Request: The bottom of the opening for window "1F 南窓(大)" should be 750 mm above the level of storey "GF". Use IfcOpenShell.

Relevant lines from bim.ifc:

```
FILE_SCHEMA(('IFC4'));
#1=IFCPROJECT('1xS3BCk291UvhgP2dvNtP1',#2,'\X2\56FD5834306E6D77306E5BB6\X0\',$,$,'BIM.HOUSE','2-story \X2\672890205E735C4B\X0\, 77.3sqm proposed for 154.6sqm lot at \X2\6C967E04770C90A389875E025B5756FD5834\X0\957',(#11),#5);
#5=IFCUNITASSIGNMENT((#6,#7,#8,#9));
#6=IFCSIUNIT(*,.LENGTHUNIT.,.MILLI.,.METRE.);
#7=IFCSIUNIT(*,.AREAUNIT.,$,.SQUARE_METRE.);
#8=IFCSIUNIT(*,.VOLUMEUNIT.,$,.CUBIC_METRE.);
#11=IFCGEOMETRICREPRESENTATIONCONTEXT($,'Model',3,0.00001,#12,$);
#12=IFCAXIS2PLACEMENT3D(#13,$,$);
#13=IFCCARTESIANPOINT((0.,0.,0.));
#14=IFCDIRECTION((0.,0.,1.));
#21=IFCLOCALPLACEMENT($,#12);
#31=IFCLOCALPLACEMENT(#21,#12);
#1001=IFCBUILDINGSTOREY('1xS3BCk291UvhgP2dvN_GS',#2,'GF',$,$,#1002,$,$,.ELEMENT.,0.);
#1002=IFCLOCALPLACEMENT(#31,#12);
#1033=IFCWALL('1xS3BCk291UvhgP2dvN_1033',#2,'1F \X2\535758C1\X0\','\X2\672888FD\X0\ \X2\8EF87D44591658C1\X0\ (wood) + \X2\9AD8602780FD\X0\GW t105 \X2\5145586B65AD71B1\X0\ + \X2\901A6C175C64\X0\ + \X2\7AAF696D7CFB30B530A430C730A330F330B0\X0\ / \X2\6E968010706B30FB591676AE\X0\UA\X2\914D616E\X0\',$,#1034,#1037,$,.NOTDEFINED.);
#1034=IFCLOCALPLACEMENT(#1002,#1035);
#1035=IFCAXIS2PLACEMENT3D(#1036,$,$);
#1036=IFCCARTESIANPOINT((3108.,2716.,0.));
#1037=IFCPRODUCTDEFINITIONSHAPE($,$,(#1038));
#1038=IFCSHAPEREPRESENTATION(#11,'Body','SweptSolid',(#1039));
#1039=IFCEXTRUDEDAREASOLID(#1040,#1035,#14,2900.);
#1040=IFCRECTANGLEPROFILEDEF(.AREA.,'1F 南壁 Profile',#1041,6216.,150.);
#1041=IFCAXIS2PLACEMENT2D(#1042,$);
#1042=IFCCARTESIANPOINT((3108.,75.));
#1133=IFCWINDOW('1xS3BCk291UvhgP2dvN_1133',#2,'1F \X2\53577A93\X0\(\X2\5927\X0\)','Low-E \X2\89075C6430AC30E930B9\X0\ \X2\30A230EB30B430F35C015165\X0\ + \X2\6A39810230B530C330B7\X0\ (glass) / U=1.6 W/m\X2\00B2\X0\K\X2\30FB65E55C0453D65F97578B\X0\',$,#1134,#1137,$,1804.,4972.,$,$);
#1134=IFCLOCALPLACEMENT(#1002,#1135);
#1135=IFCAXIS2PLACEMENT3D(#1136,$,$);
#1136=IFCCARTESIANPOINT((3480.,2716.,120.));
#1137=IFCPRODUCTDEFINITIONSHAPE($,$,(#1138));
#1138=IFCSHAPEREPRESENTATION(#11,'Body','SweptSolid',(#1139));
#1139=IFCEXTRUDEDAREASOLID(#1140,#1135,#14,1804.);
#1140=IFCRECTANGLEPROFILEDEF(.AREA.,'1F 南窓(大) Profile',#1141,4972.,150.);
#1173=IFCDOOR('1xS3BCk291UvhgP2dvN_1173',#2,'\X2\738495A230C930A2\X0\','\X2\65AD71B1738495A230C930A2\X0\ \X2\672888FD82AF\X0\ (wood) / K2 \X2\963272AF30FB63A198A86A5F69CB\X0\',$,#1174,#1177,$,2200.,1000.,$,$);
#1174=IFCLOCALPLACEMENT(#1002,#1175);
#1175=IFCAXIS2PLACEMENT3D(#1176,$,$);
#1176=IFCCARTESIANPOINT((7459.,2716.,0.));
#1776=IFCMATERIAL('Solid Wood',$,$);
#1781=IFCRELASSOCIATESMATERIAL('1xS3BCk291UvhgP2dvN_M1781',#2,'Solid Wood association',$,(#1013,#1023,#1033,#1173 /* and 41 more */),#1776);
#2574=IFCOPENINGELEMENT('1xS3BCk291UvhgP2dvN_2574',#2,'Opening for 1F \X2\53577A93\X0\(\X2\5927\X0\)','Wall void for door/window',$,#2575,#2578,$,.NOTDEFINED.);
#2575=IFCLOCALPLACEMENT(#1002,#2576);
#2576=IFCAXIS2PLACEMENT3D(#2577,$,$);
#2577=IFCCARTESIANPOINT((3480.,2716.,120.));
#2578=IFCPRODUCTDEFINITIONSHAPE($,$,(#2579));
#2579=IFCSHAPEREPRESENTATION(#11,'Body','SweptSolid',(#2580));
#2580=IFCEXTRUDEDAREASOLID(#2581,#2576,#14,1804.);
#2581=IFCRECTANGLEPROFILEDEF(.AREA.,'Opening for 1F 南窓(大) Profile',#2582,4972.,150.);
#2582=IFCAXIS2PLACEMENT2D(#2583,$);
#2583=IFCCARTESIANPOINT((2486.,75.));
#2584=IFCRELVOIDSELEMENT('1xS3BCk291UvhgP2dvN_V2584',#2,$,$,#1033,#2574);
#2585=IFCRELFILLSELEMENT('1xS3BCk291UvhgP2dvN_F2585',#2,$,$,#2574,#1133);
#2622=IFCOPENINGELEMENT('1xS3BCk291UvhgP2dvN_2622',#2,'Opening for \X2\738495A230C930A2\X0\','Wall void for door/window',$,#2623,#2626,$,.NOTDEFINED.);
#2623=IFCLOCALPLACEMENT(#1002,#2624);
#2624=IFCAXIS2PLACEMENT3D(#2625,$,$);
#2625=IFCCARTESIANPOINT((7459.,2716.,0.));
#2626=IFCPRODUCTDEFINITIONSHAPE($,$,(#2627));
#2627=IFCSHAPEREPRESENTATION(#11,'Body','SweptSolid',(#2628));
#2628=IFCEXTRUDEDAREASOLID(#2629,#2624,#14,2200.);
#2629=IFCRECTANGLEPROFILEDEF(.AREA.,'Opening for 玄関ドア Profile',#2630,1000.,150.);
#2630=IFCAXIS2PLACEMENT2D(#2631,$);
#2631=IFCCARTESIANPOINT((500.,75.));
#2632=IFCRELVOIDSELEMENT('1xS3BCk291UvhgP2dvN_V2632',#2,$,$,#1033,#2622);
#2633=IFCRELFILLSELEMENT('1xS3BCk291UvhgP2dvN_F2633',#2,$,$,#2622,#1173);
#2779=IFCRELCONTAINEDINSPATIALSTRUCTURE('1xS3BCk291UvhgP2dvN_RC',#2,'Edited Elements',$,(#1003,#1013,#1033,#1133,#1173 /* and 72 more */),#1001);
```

```python
import numpy as np
import ifcopenshell
import ifcopenshell.api.geometry
import ifcopenshell.geom
import ifcopenshell.util.element
import ifcopenshell.util.placement
import ifcopenshell.util.shape
import ifcopenshell.util.unit

model = ifcopenshell.open("bim.ifc")
unit_scale = ifcopenshell.util.unit.calculate_unit_scale(model)

window = model.by_guid("1xS3BCk291UvhgP2dvN_1133")
opening = window.FillsVoids[0].RelatingOpeningElement
storey = ifcopenshell.util.element.get_container(window, ifc_class="IfcBuildingStorey")
level = ifcopenshell.util.placement.get_local_placement(storey.ObjectPlacement)[2, 3]

# The opening's origin need not be at the sill, so measure its lowest point.
shape = ifcopenshell.geom.create_shape(ifcopenshell.geom.settings(), opening)
bottom = ifcopenshell.util.shape.get_shape_bottom_elevation(shape, shape.geometry) / unit_scale
dz = level + 0.75 / unit_scale - bottom

shift = np.array([0.0, 0.0, dz])
# The window is not placed relative to its opening, so move both.
for product in (opening, window):
    matrix = ifcopenshell.util.placement.get_local_placement(product.ObjectPlacement)
    matrix[:3, 3] += shift
    ifcopenshell.api.geometry.edit_object_placement(model, product=product, matrix=matrix, is_si=False)

print(f"moved by {dz * unit_scale:+.3f} m")

model.write("bim_v2.ifc")
```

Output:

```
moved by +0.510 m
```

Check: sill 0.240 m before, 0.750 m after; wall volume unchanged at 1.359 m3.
